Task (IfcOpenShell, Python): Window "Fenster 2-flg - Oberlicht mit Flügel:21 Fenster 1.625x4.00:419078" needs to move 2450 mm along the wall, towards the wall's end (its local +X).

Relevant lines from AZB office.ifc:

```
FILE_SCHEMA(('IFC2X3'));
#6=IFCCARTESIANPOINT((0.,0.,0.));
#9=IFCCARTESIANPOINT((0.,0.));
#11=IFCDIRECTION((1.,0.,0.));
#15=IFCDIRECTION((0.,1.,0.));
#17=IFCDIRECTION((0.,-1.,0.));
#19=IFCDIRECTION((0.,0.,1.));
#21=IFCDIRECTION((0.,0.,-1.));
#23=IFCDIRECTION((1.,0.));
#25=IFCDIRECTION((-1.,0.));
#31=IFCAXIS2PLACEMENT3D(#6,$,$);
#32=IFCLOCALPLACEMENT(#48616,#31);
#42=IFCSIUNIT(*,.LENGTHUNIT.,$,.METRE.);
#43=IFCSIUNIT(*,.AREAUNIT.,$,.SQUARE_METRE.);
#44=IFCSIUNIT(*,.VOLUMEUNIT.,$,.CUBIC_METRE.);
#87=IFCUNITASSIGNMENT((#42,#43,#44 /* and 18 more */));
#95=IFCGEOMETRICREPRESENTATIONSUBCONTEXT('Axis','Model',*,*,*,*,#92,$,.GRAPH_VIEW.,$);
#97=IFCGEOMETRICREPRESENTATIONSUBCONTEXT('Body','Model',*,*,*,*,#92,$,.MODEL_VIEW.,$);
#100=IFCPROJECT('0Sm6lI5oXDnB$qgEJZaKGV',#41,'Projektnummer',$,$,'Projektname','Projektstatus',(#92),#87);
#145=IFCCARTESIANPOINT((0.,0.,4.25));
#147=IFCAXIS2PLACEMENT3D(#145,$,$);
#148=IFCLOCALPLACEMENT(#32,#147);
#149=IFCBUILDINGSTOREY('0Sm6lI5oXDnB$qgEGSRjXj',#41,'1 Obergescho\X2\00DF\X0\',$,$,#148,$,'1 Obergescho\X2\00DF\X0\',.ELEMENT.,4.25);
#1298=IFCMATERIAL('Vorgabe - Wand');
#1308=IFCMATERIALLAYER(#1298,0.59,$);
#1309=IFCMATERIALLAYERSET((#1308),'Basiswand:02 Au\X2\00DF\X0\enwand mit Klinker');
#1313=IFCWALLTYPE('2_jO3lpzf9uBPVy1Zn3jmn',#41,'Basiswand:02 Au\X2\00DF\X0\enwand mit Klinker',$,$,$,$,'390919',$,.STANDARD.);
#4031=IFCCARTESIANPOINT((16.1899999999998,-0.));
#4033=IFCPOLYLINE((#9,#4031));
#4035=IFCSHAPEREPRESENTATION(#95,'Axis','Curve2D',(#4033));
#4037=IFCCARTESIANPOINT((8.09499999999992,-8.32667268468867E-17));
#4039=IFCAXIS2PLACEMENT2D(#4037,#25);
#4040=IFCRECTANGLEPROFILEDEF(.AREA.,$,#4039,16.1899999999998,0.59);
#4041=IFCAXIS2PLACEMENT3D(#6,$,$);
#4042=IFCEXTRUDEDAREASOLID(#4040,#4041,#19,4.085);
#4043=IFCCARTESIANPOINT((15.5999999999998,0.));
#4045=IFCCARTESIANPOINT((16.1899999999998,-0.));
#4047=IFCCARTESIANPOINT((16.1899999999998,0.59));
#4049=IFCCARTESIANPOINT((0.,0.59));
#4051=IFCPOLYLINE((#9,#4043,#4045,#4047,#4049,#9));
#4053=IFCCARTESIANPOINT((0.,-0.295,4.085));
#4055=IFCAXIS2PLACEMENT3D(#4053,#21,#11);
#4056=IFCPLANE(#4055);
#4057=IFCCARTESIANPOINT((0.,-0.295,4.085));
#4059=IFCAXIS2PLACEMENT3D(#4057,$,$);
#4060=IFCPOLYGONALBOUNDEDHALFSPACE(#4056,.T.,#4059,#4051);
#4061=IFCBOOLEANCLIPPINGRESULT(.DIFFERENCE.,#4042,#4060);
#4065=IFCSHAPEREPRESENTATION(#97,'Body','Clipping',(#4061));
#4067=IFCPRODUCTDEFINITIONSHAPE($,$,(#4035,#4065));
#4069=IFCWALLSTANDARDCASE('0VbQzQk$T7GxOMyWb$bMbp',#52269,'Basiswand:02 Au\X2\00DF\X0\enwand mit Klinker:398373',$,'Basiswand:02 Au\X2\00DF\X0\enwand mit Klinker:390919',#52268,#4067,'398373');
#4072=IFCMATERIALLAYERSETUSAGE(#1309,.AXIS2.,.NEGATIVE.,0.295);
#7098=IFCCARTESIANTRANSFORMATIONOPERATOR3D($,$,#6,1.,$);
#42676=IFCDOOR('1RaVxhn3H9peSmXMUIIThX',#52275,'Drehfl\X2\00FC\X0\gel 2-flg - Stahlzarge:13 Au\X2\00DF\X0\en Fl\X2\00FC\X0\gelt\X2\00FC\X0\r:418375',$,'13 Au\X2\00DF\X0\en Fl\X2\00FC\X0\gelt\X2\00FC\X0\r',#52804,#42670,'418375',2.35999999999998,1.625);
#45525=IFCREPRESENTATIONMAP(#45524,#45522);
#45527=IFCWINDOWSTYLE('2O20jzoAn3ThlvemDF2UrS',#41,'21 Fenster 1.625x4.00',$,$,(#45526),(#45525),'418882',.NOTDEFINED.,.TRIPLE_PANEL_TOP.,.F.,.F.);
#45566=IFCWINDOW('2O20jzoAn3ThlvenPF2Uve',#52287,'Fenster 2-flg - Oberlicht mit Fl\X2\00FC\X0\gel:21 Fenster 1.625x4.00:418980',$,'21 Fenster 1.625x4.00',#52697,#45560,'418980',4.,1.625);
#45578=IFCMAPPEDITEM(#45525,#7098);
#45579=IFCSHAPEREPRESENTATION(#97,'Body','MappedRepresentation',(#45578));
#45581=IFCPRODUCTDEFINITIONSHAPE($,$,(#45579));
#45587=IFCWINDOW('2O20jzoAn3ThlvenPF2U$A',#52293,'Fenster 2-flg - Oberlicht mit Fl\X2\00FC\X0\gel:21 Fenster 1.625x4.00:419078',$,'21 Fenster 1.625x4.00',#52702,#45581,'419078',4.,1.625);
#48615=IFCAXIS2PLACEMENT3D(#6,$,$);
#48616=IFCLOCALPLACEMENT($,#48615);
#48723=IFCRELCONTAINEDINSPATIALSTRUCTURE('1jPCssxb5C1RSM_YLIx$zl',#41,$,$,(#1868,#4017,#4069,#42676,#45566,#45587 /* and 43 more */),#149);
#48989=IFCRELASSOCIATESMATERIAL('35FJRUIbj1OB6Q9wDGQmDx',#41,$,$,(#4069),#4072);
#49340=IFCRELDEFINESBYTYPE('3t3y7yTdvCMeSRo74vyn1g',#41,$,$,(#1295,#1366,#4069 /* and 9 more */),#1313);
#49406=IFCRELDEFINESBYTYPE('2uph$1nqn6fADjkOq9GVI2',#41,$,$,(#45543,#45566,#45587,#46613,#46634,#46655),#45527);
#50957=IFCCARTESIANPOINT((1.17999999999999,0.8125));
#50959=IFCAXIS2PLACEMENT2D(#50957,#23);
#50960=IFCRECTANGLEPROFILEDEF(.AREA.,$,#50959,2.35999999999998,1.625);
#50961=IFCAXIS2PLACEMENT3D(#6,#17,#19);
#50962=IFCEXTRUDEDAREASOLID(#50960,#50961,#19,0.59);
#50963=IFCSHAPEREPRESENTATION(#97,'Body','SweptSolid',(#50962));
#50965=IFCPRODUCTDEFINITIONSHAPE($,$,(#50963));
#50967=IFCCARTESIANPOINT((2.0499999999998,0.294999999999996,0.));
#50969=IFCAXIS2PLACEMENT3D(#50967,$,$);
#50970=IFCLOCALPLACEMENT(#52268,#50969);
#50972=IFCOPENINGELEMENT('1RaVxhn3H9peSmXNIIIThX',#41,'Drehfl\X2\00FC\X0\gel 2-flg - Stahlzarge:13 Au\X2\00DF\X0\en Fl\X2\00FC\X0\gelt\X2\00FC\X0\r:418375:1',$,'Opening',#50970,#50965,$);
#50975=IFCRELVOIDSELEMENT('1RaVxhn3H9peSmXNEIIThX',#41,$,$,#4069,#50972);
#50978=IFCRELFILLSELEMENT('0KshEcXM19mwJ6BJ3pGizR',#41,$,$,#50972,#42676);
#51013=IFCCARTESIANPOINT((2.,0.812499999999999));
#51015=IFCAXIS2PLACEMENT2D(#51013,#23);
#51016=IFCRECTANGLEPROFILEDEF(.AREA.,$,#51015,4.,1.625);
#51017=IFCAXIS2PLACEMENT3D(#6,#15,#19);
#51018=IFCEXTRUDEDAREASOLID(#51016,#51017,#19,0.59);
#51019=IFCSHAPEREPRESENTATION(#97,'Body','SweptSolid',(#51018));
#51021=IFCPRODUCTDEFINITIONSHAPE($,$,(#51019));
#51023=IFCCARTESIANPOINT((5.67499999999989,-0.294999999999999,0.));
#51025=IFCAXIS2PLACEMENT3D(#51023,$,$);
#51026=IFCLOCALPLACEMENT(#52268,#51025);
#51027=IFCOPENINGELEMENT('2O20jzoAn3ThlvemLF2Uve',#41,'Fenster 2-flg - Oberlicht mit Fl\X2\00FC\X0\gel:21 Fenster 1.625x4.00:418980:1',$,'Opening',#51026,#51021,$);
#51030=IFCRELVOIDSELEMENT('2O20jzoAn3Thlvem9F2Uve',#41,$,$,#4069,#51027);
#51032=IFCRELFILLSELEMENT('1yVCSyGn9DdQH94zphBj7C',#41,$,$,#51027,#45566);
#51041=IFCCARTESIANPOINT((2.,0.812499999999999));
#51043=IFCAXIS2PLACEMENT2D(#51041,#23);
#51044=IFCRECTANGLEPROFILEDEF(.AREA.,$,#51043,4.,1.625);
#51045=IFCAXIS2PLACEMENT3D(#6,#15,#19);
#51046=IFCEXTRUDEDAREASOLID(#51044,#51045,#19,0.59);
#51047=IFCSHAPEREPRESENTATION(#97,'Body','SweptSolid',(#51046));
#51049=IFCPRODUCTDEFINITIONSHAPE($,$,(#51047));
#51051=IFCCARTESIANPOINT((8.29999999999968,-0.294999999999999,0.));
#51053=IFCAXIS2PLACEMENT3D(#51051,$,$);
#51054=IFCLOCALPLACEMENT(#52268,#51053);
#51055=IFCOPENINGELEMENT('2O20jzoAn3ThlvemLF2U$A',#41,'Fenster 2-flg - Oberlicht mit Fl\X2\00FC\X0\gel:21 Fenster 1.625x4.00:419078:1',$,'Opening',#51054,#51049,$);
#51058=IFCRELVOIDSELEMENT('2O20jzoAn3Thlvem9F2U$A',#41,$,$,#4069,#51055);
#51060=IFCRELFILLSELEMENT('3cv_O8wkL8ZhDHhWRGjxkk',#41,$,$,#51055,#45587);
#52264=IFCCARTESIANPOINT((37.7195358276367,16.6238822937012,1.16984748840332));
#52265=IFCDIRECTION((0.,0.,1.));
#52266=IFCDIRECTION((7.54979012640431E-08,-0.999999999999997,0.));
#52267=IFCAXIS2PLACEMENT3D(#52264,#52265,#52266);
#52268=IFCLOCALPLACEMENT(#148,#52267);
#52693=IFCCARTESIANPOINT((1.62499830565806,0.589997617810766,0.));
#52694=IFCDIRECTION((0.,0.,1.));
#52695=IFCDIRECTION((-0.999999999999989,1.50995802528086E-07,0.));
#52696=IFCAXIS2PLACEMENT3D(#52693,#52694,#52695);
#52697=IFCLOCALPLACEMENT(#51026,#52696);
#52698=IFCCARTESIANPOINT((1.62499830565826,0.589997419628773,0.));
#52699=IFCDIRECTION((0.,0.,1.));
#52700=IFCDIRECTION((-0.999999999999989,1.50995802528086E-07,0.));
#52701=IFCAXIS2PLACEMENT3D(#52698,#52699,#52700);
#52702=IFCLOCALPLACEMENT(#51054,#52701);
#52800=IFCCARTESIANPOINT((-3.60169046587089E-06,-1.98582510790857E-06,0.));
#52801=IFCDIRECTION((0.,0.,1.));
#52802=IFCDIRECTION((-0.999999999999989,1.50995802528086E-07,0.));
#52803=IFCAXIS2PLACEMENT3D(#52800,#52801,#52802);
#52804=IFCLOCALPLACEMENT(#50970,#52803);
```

```python
import ifcopenshell
import ifcopenshell.api.geometry
import ifcopenshell.util.placement

model = ifcopenshell.open("AZB office.ifc")

window = model.by_guid("2O20jzoAn3ThlvenPF2U$A")
opening = window.FillsVoids[0].RelatingOpeningElement
wall = opening.VoidsElements[0].RelatingBuildingElement

wall_matrix = ifcopenshell.util.placement.get_local_placement(wall.ObjectPlacement)
shift = wall_matrix[:3, 0] * 2.45
before = ifcopenshell.util.placement.get_local_placement(window.ObjectPlacement)[:3, 3].copy()

# The window is placed relative to its opening, so it follows when the opening moves.
matrix = ifcopenshell.util.placement.get_local_placement(opening.ObjectPlacement)
matrix[:3, 3] += shift
ifcopenshell.api.geometry.edit_object_placement(
    model, product=opening, matrix=matrix, is_si=False, should_transform_children=True
)

after = ifcopenshell.util.placement.get_local_placement(window.ObjectPlacement)[:3, 3]
print("window moved by", (after - before).round(3) + 0.0)

model.write("AZB office_edited.ifc")
```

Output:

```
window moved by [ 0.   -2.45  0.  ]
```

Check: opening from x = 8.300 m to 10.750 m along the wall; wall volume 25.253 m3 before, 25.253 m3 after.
